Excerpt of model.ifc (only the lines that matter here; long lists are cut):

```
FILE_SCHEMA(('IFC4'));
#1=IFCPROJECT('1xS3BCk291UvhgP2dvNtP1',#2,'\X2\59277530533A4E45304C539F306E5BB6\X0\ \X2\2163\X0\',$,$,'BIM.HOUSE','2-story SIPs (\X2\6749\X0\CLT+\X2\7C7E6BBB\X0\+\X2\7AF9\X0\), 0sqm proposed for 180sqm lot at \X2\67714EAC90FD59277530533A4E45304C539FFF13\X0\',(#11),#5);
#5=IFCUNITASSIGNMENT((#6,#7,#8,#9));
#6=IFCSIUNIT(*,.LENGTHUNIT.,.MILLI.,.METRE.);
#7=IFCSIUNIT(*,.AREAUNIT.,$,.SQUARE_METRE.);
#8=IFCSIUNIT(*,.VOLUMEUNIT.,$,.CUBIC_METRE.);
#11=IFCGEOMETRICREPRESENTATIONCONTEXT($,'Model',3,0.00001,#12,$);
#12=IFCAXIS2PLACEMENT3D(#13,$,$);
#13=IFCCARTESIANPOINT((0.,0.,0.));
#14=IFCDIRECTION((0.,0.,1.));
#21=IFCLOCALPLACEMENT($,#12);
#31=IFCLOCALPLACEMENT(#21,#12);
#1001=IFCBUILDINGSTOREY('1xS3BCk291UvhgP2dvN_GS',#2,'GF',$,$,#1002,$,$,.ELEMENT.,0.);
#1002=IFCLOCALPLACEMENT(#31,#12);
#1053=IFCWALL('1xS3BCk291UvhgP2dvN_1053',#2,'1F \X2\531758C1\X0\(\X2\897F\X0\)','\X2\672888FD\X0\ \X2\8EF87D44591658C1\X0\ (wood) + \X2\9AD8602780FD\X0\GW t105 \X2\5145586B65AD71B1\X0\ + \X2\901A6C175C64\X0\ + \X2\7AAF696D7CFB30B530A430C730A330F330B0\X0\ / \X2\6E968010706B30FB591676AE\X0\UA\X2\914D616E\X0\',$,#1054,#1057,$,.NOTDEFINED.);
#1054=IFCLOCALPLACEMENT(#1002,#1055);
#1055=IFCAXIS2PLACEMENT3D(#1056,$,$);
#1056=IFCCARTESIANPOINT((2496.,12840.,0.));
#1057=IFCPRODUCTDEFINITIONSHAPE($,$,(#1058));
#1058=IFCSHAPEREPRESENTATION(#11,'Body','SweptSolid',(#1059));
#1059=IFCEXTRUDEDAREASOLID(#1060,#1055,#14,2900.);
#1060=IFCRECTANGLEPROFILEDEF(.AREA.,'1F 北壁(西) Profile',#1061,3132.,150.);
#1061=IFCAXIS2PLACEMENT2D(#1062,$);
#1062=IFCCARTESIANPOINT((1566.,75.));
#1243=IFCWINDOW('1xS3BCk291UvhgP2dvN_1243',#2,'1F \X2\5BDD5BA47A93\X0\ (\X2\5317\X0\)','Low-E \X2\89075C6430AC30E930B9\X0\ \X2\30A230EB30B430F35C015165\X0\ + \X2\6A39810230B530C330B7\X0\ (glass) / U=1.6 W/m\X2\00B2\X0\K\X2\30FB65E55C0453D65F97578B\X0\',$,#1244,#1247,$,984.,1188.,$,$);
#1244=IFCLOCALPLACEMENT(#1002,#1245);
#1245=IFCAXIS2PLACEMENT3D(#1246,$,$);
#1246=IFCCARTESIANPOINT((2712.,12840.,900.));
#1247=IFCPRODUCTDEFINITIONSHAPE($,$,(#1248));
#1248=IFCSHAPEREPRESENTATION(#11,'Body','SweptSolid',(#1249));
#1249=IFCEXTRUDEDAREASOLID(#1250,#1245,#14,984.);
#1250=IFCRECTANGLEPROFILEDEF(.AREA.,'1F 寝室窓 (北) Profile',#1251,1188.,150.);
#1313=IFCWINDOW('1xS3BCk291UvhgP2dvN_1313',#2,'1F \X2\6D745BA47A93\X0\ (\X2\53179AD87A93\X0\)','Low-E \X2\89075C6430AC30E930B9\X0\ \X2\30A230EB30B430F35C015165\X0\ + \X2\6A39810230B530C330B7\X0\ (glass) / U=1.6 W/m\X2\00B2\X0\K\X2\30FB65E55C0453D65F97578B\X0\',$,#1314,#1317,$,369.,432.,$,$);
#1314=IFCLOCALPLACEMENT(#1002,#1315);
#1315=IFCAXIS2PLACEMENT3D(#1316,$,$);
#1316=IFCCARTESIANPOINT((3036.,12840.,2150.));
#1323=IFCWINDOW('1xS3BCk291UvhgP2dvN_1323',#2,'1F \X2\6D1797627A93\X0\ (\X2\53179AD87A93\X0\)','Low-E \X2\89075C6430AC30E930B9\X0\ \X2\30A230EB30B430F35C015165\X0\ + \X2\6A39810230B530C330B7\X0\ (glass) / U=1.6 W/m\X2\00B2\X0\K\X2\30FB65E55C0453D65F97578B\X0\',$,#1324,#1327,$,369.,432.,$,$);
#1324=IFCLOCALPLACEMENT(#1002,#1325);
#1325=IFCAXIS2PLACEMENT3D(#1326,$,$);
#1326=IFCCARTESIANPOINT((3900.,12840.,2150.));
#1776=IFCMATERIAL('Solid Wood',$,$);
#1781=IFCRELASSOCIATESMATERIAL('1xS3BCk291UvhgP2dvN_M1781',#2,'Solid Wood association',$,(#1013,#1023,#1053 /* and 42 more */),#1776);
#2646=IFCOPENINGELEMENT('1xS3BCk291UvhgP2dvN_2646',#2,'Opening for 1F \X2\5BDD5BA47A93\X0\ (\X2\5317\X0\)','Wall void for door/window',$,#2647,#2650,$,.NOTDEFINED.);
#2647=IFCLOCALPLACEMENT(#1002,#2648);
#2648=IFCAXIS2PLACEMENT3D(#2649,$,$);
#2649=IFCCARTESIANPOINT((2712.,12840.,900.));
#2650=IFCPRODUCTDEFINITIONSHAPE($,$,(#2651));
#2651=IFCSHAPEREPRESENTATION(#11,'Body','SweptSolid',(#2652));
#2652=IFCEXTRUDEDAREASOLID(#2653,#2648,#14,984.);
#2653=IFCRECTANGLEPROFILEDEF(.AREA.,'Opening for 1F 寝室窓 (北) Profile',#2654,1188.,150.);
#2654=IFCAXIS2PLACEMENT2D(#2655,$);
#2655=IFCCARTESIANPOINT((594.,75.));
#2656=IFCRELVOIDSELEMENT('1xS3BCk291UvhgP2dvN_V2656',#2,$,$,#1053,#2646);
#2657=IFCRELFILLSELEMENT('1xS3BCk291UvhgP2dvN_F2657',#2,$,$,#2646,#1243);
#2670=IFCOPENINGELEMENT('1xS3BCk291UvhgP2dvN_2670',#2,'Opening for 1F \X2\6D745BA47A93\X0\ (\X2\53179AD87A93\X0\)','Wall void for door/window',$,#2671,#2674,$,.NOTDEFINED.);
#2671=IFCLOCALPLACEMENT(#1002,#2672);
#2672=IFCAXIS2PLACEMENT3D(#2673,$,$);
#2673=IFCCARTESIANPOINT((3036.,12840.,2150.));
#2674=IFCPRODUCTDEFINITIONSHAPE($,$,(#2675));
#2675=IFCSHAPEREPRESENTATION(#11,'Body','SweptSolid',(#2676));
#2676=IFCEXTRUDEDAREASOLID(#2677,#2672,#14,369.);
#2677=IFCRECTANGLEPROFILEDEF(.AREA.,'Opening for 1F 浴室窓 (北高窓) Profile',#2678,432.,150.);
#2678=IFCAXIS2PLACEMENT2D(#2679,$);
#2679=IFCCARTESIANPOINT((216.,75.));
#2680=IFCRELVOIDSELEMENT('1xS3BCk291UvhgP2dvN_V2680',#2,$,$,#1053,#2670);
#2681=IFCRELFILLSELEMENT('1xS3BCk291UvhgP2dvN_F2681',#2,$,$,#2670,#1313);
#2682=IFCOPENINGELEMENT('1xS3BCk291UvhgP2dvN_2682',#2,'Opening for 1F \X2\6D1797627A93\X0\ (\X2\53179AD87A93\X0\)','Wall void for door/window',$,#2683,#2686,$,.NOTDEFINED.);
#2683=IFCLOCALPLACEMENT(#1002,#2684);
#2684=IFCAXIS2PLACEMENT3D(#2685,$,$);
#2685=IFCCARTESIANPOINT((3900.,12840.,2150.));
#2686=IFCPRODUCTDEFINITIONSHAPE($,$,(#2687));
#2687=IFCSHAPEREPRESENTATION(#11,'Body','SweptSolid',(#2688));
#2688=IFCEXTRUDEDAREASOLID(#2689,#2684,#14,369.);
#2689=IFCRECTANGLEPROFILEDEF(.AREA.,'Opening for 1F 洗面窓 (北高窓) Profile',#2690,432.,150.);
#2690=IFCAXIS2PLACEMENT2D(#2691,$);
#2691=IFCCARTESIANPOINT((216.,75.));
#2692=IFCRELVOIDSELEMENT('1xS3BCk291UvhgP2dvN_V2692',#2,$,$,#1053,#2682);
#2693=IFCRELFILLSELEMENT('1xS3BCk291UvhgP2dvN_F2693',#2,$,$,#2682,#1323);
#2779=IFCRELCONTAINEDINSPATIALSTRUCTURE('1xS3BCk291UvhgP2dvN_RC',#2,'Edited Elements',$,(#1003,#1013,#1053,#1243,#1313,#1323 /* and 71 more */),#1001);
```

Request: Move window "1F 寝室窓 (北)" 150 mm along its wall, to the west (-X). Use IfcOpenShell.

```python
import ifcopenshell
import ifcopenshell.api.geometry
import ifcopenshell.util.placement
import ifcopenshell.util.unit

model = ifcopenshell.open("model.ifc")
unit_scale = ifcopenshell.util.unit.calculate_unit_scale(model)

window = model.by_guid("1xS3BCk291UvhgP2dvN_1243")
opening = window.FillsVoids[0].RelatingOpeningElement
wall = opening.VoidsElements[0].RelatingBuildingElement

wall_matrix = ifcopenshell.util.placement.get_local_placement(wall.ObjectPlacement)
shift = wall_matrix[:3, 0] * -0.15 / unit_scale
before = ifcopenshell.util.placement.get_local_placement(window.ObjectPlacement)[:3, 3].copy()

# The window is not placed relative to its opening, so move both.
for product in (opening, window):
    matrix = ifcopenshell.util.placement.get_local_placement(product.ObjectPlacement)
    matrix[:3, 3] += shift
    ifcopenshell.api.geometry.edit_object_placement(model, product=product, matrix=matrix, is_si=False)

after = ifcopenshell.util.placement.get_local_placement(window.ObjectPlacement)[:3, 3]
print("window moved by", (after - before).round(3) + 0.0)

model.write("model-out.ifc")
```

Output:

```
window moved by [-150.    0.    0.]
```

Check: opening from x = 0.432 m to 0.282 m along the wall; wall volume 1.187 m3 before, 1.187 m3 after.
